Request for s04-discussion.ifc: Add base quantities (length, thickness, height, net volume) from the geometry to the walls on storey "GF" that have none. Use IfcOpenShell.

First a look at what the model holds.

```python
import ifcopenshell
import ifcopenshell.util.element
import ifcopenshell.util.unit

model = ifcopenshell.open("s04-discussion.ifc")
print(model.schema)
for unit_type in ("LENGTHUNIT", "AREAUNIT", "VOLUMEUNIT"):
    print(unit_type, ifcopenshell.util.unit.calculate_unit_scale(model, unit_type))
storey = next(s for s in model.by_type("IfcBuildingStorey") if s.Name == "GF")
walls = [e for e in ifcopenshell.util.element.get_decomposition(storey) if e.is_a("IfcWall")]
for e in sorted(walls, key=lambda e: e.id()):
    print(e.id(), e.is_a(), e.Name, list(ifcopenshell.util.element.get_psets(e, qtos_only=True)), sep=" | ")
```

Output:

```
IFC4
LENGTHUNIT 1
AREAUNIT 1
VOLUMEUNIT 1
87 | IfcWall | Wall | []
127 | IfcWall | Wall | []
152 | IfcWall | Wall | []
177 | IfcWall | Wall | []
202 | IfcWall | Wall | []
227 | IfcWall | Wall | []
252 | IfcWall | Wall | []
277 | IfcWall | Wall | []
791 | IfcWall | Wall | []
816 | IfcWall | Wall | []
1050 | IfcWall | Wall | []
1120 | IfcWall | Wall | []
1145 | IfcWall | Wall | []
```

```python
import ifcopenshell
import ifcopenshell.api.pset
import ifcopenshell.geom
import ifcopenshell.util.element
import ifcopenshell.util.shape
import ifcopenshell.util.unit

model = ifcopenshell.open("s04-discussion.ifc")
unit_scale = ifcopenshell.util.unit.calculate_unit_scale(model)
volume_scale = ifcopenshell.util.unit.calculate_unit_scale(model, "VOLUMEUNIT")
settings = ifcopenshell.geom.settings()

storey = next(s for s in model.by_type("IfcBuildingStorey") if s.Name == "GF")
walls = [e for e in ifcopenshell.util.element.get_decomposition(storey) if e.is_a("IfcWall")]

for e in sorted(walls, key=lambda e: e.id()):
    if ifcopenshell.util.element.get_psets(e, qtos_only=True, should_inherit=False):
        continue
    # Geometry comes back in metres, in the element's own axes.
    shape = ifcopenshell.geom.create_shape(settings, e)
    values = {
        "Length": ifcopenshell.util.shape.get_x(shape.geometry) / unit_scale,
        "Width": ifcopenshell.util.shape.get_y(shape.geometry) / unit_scale,
        "Height": ifcopenshell.util.shape.get_z(shape.geometry) / unit_scale,
        "NetVolume": ifcopenshell.util.shape.get_volume(shape.geometry) / volume_scale,
    }
    qto = ifcopenshell.api.pset.add_qto(model, product=e, name="Qto_WallBaseQuantities")
    ifcopenshell.api.pset.edit_qto(model, qto=qto, properties=values)
    print(e.id(), {k: round(v, 3) for k, v in values.items()})

model.write("s04-discussion-out.ifc")
```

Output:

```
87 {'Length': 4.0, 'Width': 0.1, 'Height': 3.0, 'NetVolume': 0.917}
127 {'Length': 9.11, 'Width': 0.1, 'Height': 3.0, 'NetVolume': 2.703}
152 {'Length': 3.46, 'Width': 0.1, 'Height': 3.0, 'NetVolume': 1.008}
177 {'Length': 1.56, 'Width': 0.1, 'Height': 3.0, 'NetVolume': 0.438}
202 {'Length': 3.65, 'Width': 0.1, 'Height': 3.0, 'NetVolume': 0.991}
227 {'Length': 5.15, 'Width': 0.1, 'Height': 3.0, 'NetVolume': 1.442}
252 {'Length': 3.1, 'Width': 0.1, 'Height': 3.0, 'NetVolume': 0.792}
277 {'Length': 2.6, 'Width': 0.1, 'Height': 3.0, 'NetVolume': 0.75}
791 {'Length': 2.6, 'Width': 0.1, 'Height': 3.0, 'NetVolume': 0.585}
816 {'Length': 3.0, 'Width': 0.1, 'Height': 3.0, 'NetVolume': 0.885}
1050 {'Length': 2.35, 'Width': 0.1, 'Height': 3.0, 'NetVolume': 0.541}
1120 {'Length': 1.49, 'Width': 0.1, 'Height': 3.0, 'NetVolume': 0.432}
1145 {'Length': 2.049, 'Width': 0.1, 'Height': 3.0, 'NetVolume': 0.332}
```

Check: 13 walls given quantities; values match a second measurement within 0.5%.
